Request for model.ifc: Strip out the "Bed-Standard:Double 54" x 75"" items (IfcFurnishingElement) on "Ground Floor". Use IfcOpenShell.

First a look at what the model holds.

```python
import ifcopenshell
import ifcopenshell.util.element

model = ifcopenshell.open("model.ifc")
print(model.schema)
storey = next(s for s in model.by_type("IfcBuildingStorey") if s.Name == "Ground Floor")
furniture = [e for e in ifcopenshell.util.element.get_decomposition(storey) if e.is_a("IfcFurnishingElement")]
seen = {}
for e in furniture:
    element_type = ifcopenshell.util.element.get_type(e)
    name = element_type.Name if element_type not in (None, e) else None
    seen[name] = seen.get(name, 0) + 1
for name, count in sorted(seen.items(), key=str):
    print(count, "x", name)
```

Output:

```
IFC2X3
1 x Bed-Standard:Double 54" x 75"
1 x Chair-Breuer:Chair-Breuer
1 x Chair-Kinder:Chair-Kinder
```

```python
import ifcopenshell
import ifcopenshell.api.root
import ifcopenshell.util.element

model = ifcopenshell.open("model.ifc")

storey = next(s for s in model.by_type("IfcBuildingStorey") if s.Name == "Ground Floor")
furniture = [e for e in ifcopenshell.util.element.get_decomposition(storey) if e.is_a("IfcFurnishingElement")]
targets = [e for e in furniture if (t := ifcopenshell.util.element.get_type(e)) not in (None, e) and t.Name == 'Bed-Standard:Double 54" x 75"']

for e in targets:
    ifcopenshell.api.root.remove_product(model, product=e)
print(len(targets), "removed")

model.write("model-out.ifc")
```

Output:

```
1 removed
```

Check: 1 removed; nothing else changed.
